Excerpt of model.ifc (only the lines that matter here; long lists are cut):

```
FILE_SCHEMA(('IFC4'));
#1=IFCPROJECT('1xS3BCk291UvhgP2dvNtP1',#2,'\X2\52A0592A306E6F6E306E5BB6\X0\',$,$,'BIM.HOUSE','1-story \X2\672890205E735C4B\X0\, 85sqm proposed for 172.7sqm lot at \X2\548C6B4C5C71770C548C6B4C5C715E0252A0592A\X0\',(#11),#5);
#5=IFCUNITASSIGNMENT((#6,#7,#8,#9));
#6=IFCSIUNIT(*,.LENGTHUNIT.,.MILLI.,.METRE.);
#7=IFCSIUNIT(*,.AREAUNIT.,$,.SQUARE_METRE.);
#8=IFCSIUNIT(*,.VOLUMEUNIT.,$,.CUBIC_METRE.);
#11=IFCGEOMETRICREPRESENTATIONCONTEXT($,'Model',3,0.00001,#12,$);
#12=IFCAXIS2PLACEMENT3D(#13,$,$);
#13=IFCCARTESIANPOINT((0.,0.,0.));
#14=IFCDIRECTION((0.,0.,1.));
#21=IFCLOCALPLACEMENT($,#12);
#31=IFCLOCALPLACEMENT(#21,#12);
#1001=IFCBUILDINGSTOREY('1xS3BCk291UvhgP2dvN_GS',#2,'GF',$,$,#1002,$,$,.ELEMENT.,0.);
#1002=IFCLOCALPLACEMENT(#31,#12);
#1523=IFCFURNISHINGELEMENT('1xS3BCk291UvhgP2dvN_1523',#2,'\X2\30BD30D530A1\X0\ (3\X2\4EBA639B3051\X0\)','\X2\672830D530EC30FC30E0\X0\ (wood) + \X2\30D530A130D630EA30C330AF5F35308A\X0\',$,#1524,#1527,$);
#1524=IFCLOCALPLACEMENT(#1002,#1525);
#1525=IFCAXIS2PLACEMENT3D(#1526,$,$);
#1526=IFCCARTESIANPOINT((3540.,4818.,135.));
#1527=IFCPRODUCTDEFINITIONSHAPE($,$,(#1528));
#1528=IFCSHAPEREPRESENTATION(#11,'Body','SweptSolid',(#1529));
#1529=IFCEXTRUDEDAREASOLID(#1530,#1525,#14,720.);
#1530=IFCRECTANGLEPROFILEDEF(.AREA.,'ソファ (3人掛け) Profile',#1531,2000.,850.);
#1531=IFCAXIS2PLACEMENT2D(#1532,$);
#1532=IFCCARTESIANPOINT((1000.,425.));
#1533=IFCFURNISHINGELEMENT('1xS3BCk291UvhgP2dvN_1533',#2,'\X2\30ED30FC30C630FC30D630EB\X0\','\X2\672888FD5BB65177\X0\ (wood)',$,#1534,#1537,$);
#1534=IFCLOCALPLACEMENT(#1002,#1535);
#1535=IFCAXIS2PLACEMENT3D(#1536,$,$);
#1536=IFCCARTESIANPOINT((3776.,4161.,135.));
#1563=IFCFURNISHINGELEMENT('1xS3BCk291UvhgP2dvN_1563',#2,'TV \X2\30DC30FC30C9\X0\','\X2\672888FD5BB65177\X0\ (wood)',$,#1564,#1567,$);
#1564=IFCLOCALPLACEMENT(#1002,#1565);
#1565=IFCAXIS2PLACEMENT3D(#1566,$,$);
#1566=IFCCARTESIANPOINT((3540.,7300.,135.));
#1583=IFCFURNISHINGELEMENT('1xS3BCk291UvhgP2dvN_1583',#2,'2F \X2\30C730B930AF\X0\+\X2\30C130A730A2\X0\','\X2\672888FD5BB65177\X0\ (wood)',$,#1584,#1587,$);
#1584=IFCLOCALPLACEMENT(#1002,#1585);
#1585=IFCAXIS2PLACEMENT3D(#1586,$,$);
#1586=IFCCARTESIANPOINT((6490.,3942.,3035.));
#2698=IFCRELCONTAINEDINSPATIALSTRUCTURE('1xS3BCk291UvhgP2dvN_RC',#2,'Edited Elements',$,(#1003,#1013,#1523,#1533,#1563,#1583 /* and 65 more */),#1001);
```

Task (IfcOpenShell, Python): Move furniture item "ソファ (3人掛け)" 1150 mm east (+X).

```python
import ifcopenshell
import ifcopenshell.api.geometry
import ifcopenshell.util.placement
import ifcopenshell.util.unit

model = ifcopenshell.open("model.ifc")
unit_scale = ifcopenshell.util.unit.calculate_unit_scale(model)

item = model.by_guid("1xS3BCk291UvhgP2dvN_1523")
matrix = ifcopenshell.util.placement.get_local_placement(item.ObjectPlacement)
matrix[0, 3] += 1.15 / unit_scale
ifcopenshell.api.geometry.edit_object_placement(model, product=item, matrix=matrix, is_si=False)

print(ifcopenshell.util.placement.get_local_placement(item.ObjectPlacement).round(3) + 0.0)

model.write("model_edited.ifc")
```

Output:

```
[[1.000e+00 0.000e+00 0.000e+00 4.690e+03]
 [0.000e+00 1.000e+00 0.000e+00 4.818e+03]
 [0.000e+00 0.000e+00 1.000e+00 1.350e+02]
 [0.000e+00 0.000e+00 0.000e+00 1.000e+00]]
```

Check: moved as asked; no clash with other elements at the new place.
